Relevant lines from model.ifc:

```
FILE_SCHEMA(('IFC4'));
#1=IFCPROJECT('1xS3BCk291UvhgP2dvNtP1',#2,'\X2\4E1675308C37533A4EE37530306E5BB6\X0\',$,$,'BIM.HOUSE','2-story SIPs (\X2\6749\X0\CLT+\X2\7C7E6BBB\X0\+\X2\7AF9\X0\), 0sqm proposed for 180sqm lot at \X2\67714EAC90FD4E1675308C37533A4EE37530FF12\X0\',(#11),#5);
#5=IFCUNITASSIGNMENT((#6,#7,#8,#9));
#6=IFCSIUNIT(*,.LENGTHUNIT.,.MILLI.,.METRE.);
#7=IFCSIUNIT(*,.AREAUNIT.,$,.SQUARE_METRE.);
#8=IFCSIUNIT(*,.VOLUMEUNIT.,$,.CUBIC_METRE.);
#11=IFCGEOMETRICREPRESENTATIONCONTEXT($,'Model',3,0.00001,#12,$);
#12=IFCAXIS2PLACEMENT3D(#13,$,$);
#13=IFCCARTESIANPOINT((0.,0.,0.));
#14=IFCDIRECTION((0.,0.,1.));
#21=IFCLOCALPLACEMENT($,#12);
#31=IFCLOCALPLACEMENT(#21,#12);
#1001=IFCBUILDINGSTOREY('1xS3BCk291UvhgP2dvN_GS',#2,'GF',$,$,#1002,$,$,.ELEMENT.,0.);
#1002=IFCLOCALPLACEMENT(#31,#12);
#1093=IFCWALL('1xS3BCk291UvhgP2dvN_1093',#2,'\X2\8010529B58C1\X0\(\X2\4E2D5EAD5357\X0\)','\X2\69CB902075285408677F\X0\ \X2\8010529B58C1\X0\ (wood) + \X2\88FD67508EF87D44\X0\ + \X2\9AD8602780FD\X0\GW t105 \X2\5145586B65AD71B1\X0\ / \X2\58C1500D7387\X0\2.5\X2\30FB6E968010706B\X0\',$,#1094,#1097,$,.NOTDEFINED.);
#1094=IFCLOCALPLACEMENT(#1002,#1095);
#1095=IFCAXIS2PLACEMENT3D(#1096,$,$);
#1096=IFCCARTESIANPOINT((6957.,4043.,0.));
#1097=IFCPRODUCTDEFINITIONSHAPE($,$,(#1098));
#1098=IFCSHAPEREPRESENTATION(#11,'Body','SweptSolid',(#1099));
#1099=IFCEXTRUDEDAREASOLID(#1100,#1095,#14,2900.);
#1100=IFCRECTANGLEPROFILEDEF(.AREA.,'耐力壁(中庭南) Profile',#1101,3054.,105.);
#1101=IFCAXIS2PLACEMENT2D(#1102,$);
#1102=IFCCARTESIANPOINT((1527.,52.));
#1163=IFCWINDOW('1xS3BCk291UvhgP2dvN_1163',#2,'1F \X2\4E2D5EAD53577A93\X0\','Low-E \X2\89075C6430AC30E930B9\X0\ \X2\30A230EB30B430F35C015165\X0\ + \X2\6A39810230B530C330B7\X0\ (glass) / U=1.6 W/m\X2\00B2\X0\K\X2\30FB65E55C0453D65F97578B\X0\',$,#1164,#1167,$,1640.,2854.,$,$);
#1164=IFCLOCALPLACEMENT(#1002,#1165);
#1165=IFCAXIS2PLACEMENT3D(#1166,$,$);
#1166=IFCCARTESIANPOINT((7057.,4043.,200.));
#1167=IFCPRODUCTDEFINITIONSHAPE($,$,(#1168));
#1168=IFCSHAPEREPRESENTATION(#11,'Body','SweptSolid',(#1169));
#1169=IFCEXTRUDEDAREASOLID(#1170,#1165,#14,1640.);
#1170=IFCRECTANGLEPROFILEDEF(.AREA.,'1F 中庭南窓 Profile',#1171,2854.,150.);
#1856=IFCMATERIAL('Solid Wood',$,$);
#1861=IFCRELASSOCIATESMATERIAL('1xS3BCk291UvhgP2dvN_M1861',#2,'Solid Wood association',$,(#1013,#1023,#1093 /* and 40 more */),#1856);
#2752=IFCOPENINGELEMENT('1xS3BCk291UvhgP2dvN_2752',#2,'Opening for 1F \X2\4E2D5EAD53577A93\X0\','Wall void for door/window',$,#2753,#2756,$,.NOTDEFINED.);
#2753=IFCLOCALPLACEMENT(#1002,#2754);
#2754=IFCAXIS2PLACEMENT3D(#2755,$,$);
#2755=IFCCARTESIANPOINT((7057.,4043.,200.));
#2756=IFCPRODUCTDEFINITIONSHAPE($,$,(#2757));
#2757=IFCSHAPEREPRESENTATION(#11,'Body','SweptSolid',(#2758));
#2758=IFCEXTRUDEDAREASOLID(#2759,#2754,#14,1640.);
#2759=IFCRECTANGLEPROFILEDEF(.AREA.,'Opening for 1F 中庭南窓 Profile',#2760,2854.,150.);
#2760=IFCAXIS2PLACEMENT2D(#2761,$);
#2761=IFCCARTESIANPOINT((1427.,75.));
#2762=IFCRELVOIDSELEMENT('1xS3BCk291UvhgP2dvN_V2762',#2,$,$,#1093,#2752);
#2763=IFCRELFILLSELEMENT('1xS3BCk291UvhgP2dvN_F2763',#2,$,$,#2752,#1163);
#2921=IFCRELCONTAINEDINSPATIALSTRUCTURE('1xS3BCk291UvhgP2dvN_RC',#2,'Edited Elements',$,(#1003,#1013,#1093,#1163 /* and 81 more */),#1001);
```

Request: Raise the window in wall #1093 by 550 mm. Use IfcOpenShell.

```python
import numpy as np
import ifcopenshell
import ifcopenshell.api.geometry
import ifcopenshell.util.placement
import ifcopenshell.util.unit

model = ifcopenshell.open("model.ifc")
unit_scale = ifcopenshell.util.unit.calculate_unit_scale(model)

window = model.by_guid("1xS3BCk291UvhgP2dvN_1163")
opening = window.FillsVoids[0].RelatingOpeningElement
dz = 0.55 / unit_scale

shift = np.array([0.0, 0.0, dz])
# The window is not placed relative to its opening, so move both.
for product in (opening, window):
    matrix = ifcopenshell.util.placement.get_local_placement(product.ObjectPlacement)
    matrix[:3, 3] += shift
    ifcopenshell.api.geometry.edit_object_placement(model, product=product, matrix=matrix, is_si=False)

print(f"moved by {dz * unit_scale:+.3f} m")

model.write("model_rev.ifc")
```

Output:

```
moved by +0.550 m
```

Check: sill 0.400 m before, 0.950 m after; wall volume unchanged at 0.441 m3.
